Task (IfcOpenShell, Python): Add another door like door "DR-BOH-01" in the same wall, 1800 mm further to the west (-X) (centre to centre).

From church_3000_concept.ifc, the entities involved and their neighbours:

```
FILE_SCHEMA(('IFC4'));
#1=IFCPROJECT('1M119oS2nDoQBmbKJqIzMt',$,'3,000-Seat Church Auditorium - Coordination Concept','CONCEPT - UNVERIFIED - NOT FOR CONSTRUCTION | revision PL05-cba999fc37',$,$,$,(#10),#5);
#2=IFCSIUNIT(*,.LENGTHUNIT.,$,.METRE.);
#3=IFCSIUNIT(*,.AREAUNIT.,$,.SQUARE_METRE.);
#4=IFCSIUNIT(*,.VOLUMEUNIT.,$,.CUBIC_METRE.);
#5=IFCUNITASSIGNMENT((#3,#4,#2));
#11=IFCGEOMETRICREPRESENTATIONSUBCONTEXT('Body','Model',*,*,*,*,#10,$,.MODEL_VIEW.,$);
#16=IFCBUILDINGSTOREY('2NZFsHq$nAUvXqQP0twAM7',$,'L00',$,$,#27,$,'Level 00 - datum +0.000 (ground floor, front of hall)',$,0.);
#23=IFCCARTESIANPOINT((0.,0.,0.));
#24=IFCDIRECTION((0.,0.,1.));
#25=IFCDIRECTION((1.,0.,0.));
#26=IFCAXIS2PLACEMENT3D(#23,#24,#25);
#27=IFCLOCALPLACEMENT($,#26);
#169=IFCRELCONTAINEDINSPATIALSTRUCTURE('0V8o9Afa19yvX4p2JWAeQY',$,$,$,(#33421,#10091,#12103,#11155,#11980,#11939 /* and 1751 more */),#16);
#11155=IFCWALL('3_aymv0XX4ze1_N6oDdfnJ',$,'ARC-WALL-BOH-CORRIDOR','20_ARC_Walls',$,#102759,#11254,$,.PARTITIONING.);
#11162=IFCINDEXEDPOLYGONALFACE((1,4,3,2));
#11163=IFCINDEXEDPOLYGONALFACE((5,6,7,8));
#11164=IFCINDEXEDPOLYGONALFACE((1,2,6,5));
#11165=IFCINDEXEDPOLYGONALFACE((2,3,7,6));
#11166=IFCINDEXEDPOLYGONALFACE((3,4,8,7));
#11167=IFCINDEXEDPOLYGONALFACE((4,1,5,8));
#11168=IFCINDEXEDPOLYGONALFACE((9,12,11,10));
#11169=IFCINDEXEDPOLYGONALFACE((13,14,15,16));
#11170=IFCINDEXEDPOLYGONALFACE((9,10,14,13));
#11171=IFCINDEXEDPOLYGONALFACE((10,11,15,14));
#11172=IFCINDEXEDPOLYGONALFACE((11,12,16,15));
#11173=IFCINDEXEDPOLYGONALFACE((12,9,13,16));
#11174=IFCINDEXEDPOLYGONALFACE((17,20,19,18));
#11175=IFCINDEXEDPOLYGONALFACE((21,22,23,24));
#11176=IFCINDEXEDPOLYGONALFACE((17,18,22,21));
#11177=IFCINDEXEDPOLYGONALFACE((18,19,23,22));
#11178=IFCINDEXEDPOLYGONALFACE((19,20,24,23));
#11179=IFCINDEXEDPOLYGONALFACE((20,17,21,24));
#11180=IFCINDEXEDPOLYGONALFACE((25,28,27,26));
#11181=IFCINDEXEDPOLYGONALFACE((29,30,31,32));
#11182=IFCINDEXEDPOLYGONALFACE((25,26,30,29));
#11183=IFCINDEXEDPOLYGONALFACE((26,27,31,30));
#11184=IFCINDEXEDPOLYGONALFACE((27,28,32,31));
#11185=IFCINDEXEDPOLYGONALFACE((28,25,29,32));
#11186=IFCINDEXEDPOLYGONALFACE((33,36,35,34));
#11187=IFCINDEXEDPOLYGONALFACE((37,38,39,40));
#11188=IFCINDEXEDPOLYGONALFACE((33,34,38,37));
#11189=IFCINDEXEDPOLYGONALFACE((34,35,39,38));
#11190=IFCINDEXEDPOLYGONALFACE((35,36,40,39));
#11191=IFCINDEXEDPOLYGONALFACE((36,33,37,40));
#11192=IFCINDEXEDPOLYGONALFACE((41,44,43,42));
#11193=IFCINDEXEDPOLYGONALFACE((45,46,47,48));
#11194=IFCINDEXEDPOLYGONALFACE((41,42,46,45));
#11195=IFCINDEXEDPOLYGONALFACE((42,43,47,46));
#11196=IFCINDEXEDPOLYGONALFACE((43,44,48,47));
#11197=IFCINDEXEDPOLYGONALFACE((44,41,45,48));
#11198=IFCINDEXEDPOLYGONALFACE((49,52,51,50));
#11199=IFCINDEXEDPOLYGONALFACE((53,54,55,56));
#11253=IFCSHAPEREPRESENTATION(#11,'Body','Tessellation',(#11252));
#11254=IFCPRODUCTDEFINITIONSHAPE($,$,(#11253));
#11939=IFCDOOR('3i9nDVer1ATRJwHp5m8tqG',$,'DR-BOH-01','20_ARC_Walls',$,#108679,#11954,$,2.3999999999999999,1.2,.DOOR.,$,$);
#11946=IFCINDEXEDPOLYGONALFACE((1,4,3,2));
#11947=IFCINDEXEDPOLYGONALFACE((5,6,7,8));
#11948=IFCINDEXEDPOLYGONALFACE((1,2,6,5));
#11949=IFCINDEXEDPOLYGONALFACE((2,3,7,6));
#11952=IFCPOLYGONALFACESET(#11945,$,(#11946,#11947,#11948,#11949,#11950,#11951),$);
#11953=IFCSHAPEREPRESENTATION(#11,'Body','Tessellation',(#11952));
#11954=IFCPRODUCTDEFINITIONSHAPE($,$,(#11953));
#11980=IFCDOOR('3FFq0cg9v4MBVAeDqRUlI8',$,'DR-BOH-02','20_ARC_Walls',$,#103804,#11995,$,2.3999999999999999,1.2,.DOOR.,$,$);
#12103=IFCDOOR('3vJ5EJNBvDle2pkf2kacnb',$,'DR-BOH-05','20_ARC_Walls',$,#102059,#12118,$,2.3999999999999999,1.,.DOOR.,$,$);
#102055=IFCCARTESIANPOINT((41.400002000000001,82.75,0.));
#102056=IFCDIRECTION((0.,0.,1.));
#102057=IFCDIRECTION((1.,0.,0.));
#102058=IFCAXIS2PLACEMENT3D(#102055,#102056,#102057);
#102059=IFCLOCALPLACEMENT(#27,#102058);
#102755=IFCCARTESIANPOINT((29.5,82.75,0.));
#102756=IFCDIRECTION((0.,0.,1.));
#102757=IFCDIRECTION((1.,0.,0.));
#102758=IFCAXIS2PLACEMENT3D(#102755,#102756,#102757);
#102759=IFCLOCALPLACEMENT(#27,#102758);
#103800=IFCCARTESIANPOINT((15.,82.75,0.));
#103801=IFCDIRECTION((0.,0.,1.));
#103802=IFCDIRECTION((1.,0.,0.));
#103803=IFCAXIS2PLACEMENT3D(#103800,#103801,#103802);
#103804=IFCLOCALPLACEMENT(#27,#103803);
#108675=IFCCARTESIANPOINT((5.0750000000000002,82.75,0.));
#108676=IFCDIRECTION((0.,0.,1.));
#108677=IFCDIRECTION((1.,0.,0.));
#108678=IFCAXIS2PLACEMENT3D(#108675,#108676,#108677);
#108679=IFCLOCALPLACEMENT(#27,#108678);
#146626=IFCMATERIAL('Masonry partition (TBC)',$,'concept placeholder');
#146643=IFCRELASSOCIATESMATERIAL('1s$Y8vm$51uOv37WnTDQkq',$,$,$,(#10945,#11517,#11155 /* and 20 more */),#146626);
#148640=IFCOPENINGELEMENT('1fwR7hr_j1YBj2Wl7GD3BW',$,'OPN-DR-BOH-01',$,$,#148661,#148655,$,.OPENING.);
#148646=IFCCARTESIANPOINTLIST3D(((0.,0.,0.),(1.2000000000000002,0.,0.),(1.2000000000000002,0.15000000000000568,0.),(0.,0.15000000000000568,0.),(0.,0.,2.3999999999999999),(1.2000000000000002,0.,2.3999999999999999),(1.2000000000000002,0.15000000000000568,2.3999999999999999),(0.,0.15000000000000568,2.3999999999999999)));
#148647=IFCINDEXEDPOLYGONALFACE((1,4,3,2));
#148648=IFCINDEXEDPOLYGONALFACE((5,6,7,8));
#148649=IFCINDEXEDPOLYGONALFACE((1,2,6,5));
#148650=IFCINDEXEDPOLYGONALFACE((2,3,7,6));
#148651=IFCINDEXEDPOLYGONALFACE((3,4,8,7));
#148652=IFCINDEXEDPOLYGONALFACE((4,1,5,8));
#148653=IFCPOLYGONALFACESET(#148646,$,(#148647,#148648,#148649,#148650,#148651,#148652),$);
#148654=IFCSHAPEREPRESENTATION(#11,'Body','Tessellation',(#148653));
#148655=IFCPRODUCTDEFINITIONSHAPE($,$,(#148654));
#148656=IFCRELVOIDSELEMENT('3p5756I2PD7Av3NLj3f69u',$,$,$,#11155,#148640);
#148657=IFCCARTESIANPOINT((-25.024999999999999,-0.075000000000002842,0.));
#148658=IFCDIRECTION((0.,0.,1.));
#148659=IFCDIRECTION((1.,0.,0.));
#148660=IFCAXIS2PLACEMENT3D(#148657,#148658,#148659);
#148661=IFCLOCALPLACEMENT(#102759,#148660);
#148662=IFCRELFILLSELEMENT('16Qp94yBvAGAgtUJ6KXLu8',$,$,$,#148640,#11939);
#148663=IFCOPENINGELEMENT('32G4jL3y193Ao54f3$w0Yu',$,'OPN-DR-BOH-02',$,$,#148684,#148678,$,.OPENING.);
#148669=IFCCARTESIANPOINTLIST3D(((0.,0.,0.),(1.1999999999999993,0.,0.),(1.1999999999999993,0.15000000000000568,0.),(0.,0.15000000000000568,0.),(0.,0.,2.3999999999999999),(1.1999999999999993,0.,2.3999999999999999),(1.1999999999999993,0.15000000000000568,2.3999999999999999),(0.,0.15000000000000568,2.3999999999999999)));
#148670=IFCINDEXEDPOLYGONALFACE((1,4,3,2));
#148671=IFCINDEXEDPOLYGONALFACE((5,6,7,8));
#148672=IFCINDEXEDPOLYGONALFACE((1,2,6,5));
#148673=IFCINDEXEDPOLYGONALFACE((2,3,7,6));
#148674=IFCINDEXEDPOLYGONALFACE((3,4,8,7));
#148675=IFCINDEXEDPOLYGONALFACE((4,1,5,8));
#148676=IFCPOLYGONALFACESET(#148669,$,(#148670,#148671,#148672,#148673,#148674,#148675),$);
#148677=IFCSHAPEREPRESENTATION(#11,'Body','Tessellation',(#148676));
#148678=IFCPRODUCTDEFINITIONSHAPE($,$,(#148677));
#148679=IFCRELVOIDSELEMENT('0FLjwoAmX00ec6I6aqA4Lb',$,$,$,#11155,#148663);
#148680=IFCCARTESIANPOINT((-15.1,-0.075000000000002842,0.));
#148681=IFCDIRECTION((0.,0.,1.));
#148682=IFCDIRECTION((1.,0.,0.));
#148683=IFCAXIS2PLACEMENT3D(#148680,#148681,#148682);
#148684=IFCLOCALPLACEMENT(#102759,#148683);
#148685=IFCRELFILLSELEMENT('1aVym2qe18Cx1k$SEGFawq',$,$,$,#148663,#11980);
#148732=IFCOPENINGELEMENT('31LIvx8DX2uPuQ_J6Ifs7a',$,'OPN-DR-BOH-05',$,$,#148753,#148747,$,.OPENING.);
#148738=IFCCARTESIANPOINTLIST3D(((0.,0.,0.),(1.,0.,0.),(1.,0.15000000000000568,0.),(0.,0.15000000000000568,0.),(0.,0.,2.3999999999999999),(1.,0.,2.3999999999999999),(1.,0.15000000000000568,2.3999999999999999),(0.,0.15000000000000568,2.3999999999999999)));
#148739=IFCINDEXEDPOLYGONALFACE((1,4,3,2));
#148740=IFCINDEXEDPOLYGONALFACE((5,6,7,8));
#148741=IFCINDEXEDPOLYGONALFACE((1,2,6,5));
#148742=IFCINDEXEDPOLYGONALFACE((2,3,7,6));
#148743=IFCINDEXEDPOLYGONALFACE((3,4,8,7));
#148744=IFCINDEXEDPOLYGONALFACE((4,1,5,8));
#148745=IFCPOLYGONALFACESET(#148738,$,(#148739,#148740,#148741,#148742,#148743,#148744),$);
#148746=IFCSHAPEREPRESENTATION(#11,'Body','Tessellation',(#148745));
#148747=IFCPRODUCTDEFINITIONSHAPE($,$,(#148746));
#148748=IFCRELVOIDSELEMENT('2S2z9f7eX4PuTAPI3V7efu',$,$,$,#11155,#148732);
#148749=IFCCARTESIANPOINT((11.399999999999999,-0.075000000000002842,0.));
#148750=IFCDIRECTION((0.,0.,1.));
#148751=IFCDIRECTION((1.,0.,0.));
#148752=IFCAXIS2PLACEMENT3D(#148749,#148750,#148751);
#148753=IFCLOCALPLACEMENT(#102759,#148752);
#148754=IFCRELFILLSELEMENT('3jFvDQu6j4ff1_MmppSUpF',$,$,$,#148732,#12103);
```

```python
import ifcopenshell
import ifcopenshell.api.feature
import ifcopenshell.api.geometry
import ifcopenshell.api.root
import ifcopenshell.geom
import ifcopenshell.util.element
import ifcopenshell.util.placement
import ifcopenshell.util.shape
import ifcopenshell.util.unit

model = ifcopenshell.open("church_3000_concept.ifc")
unit_scale = ifcopenshell.util.unit.calculate_unit_scale(model)
settings = ifcopenshell.geom.settings()


def volume(element):
    """Net volume in cubic metres, openings subtracted."""
    shape = ifcopenshell.geom.create_shape(settings, element)
    return ifcopenshell.util.shape.get_volume(shape.geometry)


door = model.by_guid("3i9nDVer1ATRJwHp5m8tqG")
opening = door.FillsVoids[0].RelatingOpeningElement
wall = opening.VoidsElements[0].RelatingBuildingElement
before = volume(wall)
shift = ifcopenshell.util.placement.get_local_placement(wall.ObjectPlacement)[:3, 0] * -1.8 / unit_scale

# copy_class copies the void relationship, type, container and properties, but no geometry.
new_opening = ifcopenshell.api.root.copy_class(model, product=opening)
new_opening.Representation = ifcopenshell.util.element.copy_deep(
    model, opening.Representation, exclude=["IfcGeometricRepresentationContext", "IfcRepresentationMap"]
)
new_door = ifcopenshell.api.root.copy_class(model, product=door)
new_door.Representation = ifcopenshell.util.element.copy_deep(
    model, door.Representation, exclude=["IfcGeometricRepresentationContext", "IfcRepresentationMap"]
)
ifcopenshell.api.feature.add_filling(model, opening=new_opening, element=new_door)

for old, new in ((opening, new_opening), (door, new_door)):
    matrix = ifcopenshell.util.placement.get_local_placement(old.ObjectPlacement)
    matrix[:3, 3] += shift
    ifcopenshell.api.geometry.edit_object_placement(model, product=new, matrix=matrix, is_si=False)

after = volume(wall)

print(f"wall volume {before:.3f} -> {after:.3f} m3")

model.write("church_3000_concept_updated.ifc")
```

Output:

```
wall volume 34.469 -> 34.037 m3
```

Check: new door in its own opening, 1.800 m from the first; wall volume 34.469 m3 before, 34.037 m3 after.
